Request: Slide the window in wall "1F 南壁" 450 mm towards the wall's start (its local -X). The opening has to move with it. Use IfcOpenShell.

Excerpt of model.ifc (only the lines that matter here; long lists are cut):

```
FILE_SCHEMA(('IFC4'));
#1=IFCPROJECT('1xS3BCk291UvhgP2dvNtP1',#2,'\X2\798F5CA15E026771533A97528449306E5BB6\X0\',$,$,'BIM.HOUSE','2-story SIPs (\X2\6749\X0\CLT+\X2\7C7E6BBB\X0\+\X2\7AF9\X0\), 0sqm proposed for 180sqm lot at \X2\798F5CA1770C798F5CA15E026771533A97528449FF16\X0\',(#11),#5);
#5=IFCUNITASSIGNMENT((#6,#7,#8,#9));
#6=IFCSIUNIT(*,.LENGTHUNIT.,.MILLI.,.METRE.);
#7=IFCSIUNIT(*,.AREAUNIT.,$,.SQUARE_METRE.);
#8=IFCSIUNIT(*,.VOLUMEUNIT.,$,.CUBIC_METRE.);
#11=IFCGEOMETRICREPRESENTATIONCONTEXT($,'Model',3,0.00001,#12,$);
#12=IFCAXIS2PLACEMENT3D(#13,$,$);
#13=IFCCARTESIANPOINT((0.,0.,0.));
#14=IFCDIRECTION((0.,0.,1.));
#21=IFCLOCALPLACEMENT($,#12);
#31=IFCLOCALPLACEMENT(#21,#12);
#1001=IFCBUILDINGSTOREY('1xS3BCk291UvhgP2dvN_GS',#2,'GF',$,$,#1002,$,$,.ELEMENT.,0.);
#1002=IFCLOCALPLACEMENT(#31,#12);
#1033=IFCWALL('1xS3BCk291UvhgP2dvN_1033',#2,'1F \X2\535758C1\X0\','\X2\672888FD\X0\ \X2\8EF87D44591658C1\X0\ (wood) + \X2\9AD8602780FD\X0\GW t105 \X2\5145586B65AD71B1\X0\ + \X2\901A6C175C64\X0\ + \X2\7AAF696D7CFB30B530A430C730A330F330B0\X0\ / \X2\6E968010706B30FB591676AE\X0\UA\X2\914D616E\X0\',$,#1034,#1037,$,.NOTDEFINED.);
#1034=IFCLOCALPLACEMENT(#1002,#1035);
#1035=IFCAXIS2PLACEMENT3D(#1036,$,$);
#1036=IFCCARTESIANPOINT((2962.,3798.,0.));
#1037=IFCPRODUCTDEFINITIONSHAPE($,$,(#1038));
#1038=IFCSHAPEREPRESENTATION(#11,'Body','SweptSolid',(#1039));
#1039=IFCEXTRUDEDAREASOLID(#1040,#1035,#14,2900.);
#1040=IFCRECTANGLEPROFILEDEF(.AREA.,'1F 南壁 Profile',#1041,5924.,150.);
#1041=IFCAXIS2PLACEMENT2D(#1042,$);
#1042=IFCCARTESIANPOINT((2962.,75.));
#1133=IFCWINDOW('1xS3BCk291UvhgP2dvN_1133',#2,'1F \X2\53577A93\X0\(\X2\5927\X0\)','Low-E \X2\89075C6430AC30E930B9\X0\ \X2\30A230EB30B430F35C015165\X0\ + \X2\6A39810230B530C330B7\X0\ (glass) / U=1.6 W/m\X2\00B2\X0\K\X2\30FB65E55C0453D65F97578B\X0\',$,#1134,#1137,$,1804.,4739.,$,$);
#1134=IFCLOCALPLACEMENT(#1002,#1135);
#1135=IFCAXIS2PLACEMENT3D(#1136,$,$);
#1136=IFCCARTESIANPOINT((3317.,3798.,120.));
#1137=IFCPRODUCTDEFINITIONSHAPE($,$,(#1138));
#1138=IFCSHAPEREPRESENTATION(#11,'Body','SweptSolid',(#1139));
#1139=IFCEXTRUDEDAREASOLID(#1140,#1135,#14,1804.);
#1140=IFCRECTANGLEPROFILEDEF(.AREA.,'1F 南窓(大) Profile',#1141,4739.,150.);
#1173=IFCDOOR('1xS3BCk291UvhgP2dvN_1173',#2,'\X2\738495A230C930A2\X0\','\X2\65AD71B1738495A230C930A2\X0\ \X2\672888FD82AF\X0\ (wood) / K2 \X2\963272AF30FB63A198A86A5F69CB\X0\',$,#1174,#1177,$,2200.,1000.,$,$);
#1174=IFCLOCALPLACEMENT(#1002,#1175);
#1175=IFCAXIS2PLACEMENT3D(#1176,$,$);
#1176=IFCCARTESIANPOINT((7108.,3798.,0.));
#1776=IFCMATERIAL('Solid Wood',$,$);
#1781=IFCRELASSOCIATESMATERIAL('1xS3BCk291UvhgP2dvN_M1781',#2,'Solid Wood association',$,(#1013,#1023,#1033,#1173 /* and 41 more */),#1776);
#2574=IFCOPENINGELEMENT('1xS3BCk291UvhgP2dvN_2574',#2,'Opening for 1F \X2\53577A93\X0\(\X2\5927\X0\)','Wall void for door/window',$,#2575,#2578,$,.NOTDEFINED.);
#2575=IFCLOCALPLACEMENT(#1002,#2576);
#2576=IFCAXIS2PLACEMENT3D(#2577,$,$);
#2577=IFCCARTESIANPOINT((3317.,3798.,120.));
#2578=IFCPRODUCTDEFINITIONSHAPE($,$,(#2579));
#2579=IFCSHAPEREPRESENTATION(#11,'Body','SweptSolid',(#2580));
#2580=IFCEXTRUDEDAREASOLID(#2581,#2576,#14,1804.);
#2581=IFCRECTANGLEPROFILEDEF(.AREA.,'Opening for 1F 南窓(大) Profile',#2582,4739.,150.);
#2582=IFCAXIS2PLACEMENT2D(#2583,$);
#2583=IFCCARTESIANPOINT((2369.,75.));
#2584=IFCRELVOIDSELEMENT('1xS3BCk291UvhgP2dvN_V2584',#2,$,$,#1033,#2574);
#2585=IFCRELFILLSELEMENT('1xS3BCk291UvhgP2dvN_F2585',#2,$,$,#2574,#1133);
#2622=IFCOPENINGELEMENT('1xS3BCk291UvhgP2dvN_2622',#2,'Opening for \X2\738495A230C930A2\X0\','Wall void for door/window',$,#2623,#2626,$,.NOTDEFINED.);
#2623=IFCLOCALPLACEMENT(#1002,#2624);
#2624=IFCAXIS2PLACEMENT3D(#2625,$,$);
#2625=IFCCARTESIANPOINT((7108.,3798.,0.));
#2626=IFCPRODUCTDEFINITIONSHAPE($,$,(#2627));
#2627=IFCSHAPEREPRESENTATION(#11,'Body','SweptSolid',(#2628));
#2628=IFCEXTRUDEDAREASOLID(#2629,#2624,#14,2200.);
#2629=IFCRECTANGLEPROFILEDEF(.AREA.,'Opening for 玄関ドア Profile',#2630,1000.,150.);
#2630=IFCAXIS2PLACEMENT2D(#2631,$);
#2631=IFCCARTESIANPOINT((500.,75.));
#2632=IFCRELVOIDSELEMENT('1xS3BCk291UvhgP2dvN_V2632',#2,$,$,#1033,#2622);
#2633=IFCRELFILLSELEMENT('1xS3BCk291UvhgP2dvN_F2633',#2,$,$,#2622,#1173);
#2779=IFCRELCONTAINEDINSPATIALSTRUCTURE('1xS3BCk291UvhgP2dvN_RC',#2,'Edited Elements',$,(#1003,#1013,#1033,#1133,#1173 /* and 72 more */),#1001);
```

```python
import ifcopenshell
import ifcopenshell.api.geometry
import ifcopenshell.util.placement

model = ifcopenshell.open("model.ifc")

window = model.by_guid("1xS3BCk291UvhgP2dvN_1133")
opening = window.FillsVoids[0].RelatingOpeningElement
wall = opening.VoidsElements[0].RelatingBuildingElement

wall_matrix = ifcopenshell.util.placement.get_local_placement(wall.ObjectPlacement)
shift = wall_matrix[:3, 0] * -450.0
before = ifcopenshell.util.placement.get_local_placement(window.ObjectPlacement)[:3, 3].copy()

# The window is not placed relative to its opening, so move both.
for product in (opening, window):
    matrix = ifcopenshell.util.placement.get_local_placement(product.ObjectPlacement)
    matrix[:3, 3] += shift
    ifcopenshell.api.geometry.edit_object_placement(model, product=product, matrix=matrix, is_si=False)

after = ifcopenshell.util.placement.get_local_placement(window.ObjectPlacement)[:3, 3]
print("window moved by", (after - before).round(3) + 0.0)

model.write("model_edited.ifc")
```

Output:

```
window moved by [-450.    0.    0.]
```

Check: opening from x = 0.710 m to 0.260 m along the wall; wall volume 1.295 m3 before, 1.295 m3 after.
